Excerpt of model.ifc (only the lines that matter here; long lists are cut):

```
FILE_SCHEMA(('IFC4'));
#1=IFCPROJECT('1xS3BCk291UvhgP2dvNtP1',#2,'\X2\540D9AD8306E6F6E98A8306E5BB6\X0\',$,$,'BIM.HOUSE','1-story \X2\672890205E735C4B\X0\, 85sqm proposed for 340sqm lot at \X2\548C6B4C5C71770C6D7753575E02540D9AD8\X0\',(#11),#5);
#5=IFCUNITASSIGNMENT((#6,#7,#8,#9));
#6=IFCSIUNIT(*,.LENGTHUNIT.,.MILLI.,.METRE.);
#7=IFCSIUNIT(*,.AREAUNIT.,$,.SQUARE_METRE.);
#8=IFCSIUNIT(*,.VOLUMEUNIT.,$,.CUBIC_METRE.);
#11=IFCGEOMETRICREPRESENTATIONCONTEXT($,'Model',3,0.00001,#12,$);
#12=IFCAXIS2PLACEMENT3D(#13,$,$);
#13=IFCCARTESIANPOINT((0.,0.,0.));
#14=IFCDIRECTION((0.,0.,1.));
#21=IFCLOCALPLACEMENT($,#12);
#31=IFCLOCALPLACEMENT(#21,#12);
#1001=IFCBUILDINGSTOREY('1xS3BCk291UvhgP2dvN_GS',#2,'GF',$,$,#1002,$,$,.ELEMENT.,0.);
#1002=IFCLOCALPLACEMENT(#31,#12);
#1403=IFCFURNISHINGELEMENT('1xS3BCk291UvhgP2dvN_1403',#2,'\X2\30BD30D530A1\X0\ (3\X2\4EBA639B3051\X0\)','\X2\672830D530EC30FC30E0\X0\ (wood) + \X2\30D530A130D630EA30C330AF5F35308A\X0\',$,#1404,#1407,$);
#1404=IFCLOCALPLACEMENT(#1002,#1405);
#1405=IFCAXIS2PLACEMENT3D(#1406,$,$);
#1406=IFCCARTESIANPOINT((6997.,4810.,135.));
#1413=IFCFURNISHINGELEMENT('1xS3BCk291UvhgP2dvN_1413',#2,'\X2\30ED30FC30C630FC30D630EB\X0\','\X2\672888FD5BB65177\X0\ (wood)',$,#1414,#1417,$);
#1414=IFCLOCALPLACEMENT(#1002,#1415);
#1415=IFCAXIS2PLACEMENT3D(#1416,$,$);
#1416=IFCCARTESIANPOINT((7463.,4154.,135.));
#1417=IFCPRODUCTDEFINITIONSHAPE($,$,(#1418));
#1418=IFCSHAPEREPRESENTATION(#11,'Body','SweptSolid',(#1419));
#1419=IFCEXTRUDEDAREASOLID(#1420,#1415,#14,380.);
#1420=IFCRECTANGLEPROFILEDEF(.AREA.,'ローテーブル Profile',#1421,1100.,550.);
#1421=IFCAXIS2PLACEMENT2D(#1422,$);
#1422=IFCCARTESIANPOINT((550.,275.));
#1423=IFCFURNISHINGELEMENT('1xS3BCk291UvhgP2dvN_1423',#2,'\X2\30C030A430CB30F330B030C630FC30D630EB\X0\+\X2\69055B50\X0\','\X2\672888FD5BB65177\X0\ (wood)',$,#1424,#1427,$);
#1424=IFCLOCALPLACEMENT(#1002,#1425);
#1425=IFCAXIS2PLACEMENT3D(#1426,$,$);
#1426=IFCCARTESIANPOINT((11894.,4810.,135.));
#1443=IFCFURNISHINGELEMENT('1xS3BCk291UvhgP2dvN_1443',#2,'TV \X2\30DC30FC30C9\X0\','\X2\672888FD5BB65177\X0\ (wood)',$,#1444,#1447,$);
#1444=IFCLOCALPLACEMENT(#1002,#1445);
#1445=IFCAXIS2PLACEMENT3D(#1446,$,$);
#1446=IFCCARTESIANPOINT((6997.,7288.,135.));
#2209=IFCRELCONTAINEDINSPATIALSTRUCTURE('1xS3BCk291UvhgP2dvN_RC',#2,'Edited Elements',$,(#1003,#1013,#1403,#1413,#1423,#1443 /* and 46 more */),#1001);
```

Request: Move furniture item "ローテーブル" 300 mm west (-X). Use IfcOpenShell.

```python
import ifcopenshell
import ifcopenshell.api.geometry
import ifcopenshell.util.placement
import ifcopenshell.util.unit

model = ifcopenshell.open("model.ifc")
unit_scale = ifcopenshell.util.unit.calculate_unit_scale(model)

item = model.by_guid("1xS3BCk291UvhgP2dvN_1413")
matrix = ifcopenshell.util.placement.get_local_placement(item.ObjectPlacement)
matrix[0, 3] -= 0.3 / unit_scale
ifcopenshell.api.geometry.edit_object_placement(model, product=item, matrix=matrix, is_si=False)

print(ifcopenshell.util.placement.get_local_placement(item.ObjectPlacement).round(3) + 0.0)

model.write("model_rev.ifc")
```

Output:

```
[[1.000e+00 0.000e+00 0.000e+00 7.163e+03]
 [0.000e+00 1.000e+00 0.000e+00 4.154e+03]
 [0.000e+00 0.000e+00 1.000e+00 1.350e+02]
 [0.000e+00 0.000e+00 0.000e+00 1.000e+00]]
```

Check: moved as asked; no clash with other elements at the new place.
